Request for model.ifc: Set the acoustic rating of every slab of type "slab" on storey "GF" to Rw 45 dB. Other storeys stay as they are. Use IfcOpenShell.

First a look at what the model holds.

```python
import ifcopenshell
import ifcopenshell.util.element

model = ifcopenshell.open("model.ifc")
print(model.schema)
storey = next(s for s in model.by_type("IfcBuildingStorey") if s.Name == "GF")
slabs = [e for e in ifcopenshell.util.element.get_decomposition(storey) if e.is_a("IfcSlab")]
seen = {}
for e in slabs:
    element_type = ifcopenshell.util.element.get_type(e)
    key = (element_type.Name if element_type != e and element_type else None, ifcopenshell.util.element.get_pset(e, "Pset_SlabCommon", "AcousticRating"))
    seen[key] = seen.get(key, 0) + 1
for (name, value), count in sorted(seen.items(), key=str):
    print(count, "x", name, "|", value)
```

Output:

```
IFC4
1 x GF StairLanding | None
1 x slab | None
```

```python
import ifcopenshell
import ifcopenshell.api.pset
import ifcopenshell.util.element

model = ifcopenshell.open("model.ifc")

storey = next(s for s in model.by_type("IfcBuildingStorey") if s.Name == "GF")
slabs = [e for e in ifcopenshell.util.element.get_decomposition(storey) if e.is_a("IfcSlab")]

count = 0
for e in slabs:
    element_type = ifcopenshell.util.element.get_type(e)
    if element_type in (None, e) or element_type.Name != "slab":
        continue
    # add_pset returns the element's existing set when there is one.
    pset = ifcopenshell.api.pset.add_pset(model, product=e, name="Pset_SlabCommon")
    ifcopenshell.api.pset.edit_pset(model, pset=pset, properties={"AcousticRating": "Rw 45 dB"})
    count += 1

print(count, "slabs updated")

model.write("model_edited.ifc")
```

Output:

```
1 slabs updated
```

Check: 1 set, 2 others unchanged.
